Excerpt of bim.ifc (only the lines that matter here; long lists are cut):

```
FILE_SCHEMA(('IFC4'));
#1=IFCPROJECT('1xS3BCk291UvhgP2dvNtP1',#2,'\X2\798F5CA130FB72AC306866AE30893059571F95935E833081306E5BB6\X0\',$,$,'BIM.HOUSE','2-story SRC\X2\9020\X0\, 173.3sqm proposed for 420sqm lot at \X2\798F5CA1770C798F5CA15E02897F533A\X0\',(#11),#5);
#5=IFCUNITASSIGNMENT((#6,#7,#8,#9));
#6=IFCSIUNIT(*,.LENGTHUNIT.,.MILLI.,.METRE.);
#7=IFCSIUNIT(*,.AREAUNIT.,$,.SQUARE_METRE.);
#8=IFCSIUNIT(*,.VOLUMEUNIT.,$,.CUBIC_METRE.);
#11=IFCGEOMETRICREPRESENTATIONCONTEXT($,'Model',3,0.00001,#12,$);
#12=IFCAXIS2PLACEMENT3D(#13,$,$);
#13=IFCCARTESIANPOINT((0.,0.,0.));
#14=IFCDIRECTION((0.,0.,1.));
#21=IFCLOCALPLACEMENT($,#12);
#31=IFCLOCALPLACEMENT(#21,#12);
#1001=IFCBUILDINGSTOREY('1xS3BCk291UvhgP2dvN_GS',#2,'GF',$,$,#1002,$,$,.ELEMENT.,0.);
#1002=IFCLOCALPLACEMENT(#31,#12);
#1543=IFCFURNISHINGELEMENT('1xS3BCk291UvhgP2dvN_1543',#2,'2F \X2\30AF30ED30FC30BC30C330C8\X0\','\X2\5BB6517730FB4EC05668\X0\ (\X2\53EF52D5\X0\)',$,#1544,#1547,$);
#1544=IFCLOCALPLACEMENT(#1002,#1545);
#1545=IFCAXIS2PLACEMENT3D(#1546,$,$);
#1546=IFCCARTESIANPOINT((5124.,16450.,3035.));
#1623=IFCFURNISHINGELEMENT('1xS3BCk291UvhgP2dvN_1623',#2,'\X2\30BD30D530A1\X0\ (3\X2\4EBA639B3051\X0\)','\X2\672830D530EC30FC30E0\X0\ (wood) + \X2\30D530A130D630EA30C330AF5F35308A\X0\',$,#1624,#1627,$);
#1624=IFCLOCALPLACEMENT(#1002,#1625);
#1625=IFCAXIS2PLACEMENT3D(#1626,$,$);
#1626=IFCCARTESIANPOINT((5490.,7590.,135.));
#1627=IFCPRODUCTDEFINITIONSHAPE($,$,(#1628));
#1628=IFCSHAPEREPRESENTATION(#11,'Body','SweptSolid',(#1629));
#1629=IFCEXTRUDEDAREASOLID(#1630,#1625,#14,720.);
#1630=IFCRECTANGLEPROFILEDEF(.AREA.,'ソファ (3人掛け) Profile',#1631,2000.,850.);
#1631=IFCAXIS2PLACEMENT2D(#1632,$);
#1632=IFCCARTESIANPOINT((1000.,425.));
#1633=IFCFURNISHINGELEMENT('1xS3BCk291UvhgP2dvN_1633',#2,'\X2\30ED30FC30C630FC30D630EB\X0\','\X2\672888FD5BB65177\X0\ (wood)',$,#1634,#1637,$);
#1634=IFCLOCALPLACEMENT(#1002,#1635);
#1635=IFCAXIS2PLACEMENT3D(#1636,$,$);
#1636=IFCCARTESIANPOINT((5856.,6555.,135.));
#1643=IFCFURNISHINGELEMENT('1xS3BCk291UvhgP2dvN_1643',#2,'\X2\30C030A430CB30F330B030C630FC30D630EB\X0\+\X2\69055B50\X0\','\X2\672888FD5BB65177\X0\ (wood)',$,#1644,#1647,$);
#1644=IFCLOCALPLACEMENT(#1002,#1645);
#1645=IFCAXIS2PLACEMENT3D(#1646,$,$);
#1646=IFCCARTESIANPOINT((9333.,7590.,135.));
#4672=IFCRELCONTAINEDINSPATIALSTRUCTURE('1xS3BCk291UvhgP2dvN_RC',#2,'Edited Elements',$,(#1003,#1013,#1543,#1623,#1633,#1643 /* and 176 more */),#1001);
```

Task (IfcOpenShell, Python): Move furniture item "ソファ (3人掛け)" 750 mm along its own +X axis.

```python
import ifcopenshell
import ifcopenshell.api.geometry
import ifcopenshell.util.placement
import ifcopenshell.util.unit

model = ifcopenshell.open("bim.ifc")
unit_scale = ifcopenshell.util.unit.calculate_unit_scale(model)

item = model.by_id(1623)
matrix = ifcopenshell.util.placement.get_local_placement(item.ObjectPlacement)
matrix[:3, 3] += matrix[:3, 0] * 0.75 / unit_scale
ifcopenshell.api.geometry.edit_object_placement(model, product=item, matrix=matrix, is_si=False)

print(ifcopenshell.util.placement.get_local_placement(item.ObjectPlacement).round(3) + 0.0)

model.write("bim_v2.ifc")
```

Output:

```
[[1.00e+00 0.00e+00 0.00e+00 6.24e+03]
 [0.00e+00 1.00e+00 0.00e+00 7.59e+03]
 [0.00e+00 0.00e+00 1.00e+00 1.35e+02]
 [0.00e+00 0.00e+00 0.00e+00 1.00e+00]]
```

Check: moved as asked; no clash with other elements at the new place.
